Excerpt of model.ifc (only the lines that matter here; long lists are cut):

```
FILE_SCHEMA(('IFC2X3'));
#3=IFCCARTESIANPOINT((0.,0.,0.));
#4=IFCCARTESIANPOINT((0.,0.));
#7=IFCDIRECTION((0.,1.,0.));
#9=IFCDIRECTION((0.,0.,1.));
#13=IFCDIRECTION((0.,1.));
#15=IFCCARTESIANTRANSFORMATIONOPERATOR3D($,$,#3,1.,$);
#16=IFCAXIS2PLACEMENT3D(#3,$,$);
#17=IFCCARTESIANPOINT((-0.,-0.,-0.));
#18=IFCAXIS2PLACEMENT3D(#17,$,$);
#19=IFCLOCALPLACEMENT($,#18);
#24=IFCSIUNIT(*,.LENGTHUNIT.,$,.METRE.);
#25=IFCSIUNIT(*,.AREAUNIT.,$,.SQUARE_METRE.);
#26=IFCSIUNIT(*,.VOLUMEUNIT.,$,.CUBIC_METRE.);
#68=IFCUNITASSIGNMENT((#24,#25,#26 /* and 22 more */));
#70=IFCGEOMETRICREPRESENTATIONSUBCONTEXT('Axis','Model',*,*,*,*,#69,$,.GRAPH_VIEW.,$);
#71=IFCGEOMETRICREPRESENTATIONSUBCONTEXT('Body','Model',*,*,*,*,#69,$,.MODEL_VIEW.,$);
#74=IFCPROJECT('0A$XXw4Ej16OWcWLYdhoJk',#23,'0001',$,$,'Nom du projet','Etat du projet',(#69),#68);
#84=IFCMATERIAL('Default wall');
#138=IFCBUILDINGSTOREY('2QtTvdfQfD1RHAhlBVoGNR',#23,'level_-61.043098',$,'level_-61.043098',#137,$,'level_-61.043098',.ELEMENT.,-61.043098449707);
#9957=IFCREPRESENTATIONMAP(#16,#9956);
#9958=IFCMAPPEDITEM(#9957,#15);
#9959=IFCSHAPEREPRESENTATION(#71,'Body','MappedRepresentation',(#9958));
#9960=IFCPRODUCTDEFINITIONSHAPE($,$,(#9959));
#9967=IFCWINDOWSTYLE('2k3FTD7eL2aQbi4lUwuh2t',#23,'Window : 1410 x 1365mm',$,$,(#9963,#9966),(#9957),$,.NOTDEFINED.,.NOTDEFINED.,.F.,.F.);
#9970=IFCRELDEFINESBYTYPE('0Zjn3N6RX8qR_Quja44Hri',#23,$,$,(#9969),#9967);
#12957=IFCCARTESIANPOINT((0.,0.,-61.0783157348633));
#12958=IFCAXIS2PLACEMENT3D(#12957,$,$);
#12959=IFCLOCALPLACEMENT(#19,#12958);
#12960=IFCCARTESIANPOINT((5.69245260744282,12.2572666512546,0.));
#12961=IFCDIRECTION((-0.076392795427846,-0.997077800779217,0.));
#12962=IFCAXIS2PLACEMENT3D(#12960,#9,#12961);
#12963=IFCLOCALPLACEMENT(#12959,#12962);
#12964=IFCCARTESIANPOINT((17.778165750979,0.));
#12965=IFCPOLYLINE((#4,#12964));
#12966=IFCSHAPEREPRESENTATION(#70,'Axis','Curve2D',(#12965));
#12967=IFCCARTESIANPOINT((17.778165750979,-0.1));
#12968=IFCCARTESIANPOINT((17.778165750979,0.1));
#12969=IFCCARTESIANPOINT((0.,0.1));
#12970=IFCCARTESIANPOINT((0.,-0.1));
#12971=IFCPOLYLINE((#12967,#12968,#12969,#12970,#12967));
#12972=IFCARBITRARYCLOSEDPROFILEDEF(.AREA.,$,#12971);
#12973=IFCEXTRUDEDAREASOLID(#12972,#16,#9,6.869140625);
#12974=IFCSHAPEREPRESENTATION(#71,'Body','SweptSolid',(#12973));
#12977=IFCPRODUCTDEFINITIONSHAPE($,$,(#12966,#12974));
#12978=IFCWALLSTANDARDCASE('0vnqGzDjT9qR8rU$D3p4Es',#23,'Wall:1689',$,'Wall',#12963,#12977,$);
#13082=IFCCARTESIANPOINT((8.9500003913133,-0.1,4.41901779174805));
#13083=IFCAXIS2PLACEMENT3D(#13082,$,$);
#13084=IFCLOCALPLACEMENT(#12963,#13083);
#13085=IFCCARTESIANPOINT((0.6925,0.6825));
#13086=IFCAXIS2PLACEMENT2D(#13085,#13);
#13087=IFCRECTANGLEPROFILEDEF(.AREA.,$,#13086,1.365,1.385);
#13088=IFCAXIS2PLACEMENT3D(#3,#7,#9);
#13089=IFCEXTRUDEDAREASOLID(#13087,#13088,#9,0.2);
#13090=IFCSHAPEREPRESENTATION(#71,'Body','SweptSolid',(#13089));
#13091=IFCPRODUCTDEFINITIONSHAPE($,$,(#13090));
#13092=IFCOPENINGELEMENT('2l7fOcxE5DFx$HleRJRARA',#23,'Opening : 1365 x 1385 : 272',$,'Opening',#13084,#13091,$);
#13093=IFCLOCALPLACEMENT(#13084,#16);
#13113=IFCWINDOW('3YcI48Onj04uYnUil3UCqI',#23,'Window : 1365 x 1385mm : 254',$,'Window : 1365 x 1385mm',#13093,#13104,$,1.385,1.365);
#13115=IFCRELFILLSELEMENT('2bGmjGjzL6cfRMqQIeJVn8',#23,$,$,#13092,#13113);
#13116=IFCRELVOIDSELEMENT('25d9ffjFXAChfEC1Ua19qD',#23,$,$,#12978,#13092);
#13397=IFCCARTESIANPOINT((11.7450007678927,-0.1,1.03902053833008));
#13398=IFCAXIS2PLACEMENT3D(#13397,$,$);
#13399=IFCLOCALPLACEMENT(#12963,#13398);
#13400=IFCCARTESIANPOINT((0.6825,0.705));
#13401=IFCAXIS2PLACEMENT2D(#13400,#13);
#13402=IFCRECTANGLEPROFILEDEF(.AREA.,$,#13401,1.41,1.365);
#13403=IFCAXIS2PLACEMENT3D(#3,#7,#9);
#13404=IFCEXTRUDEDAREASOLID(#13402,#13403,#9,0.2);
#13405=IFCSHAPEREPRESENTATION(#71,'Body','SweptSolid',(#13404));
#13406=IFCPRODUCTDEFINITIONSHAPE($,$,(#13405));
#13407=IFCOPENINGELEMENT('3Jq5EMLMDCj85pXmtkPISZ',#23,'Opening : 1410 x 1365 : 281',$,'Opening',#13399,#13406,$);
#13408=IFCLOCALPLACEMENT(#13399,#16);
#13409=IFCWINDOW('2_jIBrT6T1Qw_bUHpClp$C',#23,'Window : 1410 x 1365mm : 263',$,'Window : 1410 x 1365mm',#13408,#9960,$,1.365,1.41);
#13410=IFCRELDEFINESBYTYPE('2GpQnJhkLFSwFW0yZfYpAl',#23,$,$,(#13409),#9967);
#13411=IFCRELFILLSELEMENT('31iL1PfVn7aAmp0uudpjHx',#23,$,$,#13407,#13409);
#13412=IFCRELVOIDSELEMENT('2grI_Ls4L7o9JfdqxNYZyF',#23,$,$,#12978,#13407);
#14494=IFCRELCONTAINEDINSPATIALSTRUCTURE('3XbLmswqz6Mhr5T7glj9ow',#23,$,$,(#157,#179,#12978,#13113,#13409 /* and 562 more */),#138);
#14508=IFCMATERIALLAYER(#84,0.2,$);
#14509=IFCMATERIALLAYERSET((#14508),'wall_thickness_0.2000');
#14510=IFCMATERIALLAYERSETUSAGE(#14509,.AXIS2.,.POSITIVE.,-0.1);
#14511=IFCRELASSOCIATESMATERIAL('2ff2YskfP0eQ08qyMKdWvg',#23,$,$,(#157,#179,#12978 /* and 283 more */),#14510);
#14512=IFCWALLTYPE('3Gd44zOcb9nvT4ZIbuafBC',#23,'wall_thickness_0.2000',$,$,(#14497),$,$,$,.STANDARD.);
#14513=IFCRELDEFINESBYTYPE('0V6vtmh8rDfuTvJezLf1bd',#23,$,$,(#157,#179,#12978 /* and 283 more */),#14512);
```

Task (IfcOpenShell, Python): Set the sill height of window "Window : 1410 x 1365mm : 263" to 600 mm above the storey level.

```python
import numpy as np
import ifcopenshell
import ifcopenshell.api.geometry
import ifcopenshell.geom
import ifcopenshell.util.element
import ifcopenshell.util.placement
import ifcopenshell.util.shape
import ifcopenshell.util.unit

model = ifcopenshell.open("model.ifc")
unit_scale = ifcopenshell.util.unit.calculate_unit_scale(model)

window = model.by_guid("2_jIBrT6T1Qw_bUHpClp$C")
opening = window.FillsVoids[0].RelatingOpeningElement
storey = ifcopenshell.util.element.get_container(window, ifc_class="IfcBuildingStorey")
level = ifcopenshell.util.placement.get_local_placement(storey.ObjectPlacement)[2, 3]

# The opening's origin need not be at the sill, so measure its lowest point.
shape = ifcopenshell.geom.create_shape(ifcopenshell.geom.settings(), opening)
bottom = ifcopenshell.util.shape.get_shape_bottom_elevation(shape, shape.geometry) / unit_scale
dz = level + 0.6 - bottom

shift = np.array([0.0, 0.0, dz])
# The window is placed relative to its opening, so it follows when the opening moves.
matrix = ifcopenshell.util.placement.get_local_placement(opening.ObjectPlacement)
matrix[:3, 3] += shift
ifcopenshell.api.geometry.edit_object_placement(
    model, product=opening, matrix=matrix, is_si=False, should_transform_children=True
)

print(f"moved by {dz * unit_scale:+.3f} m")

model.write("model_rev.ifc")
```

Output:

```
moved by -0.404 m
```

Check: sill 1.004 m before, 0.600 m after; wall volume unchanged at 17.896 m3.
